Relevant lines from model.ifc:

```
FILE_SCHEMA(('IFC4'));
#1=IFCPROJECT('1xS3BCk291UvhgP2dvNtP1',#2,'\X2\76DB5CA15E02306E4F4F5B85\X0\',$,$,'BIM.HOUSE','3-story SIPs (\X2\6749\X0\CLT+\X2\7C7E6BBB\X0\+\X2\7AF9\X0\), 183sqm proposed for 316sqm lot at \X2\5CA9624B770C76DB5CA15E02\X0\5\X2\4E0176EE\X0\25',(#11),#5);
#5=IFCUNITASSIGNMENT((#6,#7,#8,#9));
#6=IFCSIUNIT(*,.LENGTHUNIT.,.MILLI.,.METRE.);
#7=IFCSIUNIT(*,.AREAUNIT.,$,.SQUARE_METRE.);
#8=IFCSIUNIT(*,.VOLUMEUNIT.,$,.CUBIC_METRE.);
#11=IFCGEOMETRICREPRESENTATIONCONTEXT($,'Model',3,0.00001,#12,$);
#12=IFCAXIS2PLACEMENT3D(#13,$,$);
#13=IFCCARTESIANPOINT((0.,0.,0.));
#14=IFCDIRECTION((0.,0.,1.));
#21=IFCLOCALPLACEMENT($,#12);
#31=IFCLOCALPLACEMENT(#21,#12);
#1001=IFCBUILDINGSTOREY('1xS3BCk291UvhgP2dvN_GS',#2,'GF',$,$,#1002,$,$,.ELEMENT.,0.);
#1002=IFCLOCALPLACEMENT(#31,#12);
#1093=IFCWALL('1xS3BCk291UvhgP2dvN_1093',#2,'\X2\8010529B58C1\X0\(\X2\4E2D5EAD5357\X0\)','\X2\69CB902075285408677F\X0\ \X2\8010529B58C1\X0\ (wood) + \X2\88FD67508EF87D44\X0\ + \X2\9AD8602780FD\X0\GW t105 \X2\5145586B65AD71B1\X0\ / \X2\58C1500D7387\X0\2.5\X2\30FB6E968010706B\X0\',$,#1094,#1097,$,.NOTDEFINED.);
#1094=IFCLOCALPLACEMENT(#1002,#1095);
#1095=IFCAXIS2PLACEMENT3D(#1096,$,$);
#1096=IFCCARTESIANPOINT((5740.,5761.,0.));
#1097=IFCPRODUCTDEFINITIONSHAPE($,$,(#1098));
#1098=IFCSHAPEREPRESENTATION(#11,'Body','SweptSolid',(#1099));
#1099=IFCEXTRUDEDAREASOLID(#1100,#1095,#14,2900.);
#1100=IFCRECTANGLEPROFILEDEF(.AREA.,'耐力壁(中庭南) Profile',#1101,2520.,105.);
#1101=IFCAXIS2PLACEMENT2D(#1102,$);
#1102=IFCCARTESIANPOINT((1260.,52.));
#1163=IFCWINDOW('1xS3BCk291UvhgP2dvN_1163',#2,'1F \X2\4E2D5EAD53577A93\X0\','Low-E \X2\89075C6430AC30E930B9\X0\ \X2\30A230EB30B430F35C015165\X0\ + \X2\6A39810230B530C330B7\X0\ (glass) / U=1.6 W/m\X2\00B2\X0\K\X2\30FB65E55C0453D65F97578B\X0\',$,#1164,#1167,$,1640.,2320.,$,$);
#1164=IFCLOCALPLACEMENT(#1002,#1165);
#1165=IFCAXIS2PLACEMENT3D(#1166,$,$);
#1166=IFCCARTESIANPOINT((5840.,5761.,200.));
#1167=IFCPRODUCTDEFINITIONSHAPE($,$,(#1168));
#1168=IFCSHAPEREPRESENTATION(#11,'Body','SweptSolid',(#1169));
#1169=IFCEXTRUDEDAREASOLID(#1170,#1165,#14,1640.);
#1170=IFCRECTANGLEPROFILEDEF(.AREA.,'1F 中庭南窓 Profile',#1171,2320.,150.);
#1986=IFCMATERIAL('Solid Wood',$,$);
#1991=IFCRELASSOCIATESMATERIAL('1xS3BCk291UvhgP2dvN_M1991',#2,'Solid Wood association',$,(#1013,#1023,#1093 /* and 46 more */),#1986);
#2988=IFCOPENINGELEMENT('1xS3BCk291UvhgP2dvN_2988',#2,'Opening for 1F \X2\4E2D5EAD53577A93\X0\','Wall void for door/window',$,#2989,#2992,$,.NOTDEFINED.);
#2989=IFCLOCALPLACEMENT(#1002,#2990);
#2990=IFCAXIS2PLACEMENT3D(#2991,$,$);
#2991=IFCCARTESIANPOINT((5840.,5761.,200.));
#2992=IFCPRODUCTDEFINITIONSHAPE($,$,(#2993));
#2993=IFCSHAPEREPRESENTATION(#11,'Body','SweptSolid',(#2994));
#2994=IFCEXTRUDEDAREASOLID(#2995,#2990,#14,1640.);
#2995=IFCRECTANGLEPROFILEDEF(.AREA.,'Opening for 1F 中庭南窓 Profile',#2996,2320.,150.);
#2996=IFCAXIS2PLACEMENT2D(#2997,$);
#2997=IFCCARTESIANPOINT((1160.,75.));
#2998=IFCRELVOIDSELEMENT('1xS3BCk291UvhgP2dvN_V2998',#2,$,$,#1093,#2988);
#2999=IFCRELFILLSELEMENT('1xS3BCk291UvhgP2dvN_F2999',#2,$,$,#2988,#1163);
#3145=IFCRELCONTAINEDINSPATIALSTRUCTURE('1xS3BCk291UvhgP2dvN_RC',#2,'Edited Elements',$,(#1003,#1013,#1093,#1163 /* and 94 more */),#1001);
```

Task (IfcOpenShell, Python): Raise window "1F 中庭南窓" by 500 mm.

```python
import numpy as np
import ifcopenshell
import ifcopenshell.api.geometry
import ifcopenshell.util.placement
import ifcopenshell.util.unit

model = ifcopenshell.open("model.ifc")
unit_scale = ifcopenshell.util.unit.calculate_unit_scale(model)

window = model.by_id(1163)
opening = window.FillsVoids[0].RelatingOpeningElement
dz = 0.5 / unit_scale

shift = np.array([0.0, 0.0, dz])
# The window is not placed relative to its opening, so move both.
for product in (opening, window):
    matrix = ifcopenshell.util.placement.get_local_placement(product.ObjectPlacement)
    matrix[:3, 3] += shift
    ifcopenshell.api.geometry.edit_object_placement(model, product=product, matrix=matrix, is_si=False)

print(f"moved by {dz * unit_scale:+.3f} m")

model.write("model_v2.ifc")
```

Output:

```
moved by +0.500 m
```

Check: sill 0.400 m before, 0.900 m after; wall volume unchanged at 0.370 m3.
